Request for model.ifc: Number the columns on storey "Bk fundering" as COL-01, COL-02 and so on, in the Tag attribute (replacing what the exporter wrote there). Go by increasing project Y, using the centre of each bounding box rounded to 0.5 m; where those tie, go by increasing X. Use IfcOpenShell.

First a look at what the model holds.

```python
import ifcopenshell
import ifcopenshell.util.element
import ifcopenshell.util.placement

model = ifcopenshell.open("model.ifc")
print(model.schema)
storey = next(s for s in model.by_type("IfcBuildingStorey") if s.Name == "Bk fundering")
columns = [e for e in ifcopenshell.util.element.get_decomposition(storey) if e.is_a("IfcColumn")]
for e in sorted(columns, key=lambda e: e.id()):
    origin = ifcopenshell.util.placement.get_local_placement(e.ObjectPlacement)[:3, 3]
    print(e.id(), e.Tag, e.Name, origin.round(2) + 0.0, sep=" | ")
```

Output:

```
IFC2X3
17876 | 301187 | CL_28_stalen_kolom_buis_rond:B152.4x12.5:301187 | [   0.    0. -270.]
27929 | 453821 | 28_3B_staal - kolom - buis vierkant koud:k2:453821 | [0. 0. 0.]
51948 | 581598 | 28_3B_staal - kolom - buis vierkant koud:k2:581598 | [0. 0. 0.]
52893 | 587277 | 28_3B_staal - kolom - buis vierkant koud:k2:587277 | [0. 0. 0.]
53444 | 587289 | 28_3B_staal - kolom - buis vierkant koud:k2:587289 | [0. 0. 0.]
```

```python
import ifcopenshell
import ifcopenshell.geom
import ifcopenshell.util.element
import ifcopenshell.util.shape

model = ifcopenshell.open("model.ifc")
settings = ifcopenshell.geom.settings()
settings.set("use-world-coords", True)


def centre(element):
    shape = ifcopenshell.geom.create_shape(settings, element)
    return ifcopenshell.util.shape.get_bbox_centroid(shape.geometry)


storey = next(s for s in model.by_type("IfcBuildingStorey") if s.Name == "Bk fundering")
columns = [e for e in ifcopenshell.util.element.get_decomposition(storey) if e.is_a("IfcColumn")]

# Insertion points can sit at a corner or the storey origin, so sort by the geometry (in metres).
centres = {e: centre(e) for e in columns}
columns.sort(key=lambda e: (round(centres[e][1] / 0.5), centres[e][0]))

for i, e in enumerate(columns, start=1):
    number = f"COL-{i:02d}"
    e.Tag = number
    print(e.id(), number)

model.write("model_rev.ifc")
```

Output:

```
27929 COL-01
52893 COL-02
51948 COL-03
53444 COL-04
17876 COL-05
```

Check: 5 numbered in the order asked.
